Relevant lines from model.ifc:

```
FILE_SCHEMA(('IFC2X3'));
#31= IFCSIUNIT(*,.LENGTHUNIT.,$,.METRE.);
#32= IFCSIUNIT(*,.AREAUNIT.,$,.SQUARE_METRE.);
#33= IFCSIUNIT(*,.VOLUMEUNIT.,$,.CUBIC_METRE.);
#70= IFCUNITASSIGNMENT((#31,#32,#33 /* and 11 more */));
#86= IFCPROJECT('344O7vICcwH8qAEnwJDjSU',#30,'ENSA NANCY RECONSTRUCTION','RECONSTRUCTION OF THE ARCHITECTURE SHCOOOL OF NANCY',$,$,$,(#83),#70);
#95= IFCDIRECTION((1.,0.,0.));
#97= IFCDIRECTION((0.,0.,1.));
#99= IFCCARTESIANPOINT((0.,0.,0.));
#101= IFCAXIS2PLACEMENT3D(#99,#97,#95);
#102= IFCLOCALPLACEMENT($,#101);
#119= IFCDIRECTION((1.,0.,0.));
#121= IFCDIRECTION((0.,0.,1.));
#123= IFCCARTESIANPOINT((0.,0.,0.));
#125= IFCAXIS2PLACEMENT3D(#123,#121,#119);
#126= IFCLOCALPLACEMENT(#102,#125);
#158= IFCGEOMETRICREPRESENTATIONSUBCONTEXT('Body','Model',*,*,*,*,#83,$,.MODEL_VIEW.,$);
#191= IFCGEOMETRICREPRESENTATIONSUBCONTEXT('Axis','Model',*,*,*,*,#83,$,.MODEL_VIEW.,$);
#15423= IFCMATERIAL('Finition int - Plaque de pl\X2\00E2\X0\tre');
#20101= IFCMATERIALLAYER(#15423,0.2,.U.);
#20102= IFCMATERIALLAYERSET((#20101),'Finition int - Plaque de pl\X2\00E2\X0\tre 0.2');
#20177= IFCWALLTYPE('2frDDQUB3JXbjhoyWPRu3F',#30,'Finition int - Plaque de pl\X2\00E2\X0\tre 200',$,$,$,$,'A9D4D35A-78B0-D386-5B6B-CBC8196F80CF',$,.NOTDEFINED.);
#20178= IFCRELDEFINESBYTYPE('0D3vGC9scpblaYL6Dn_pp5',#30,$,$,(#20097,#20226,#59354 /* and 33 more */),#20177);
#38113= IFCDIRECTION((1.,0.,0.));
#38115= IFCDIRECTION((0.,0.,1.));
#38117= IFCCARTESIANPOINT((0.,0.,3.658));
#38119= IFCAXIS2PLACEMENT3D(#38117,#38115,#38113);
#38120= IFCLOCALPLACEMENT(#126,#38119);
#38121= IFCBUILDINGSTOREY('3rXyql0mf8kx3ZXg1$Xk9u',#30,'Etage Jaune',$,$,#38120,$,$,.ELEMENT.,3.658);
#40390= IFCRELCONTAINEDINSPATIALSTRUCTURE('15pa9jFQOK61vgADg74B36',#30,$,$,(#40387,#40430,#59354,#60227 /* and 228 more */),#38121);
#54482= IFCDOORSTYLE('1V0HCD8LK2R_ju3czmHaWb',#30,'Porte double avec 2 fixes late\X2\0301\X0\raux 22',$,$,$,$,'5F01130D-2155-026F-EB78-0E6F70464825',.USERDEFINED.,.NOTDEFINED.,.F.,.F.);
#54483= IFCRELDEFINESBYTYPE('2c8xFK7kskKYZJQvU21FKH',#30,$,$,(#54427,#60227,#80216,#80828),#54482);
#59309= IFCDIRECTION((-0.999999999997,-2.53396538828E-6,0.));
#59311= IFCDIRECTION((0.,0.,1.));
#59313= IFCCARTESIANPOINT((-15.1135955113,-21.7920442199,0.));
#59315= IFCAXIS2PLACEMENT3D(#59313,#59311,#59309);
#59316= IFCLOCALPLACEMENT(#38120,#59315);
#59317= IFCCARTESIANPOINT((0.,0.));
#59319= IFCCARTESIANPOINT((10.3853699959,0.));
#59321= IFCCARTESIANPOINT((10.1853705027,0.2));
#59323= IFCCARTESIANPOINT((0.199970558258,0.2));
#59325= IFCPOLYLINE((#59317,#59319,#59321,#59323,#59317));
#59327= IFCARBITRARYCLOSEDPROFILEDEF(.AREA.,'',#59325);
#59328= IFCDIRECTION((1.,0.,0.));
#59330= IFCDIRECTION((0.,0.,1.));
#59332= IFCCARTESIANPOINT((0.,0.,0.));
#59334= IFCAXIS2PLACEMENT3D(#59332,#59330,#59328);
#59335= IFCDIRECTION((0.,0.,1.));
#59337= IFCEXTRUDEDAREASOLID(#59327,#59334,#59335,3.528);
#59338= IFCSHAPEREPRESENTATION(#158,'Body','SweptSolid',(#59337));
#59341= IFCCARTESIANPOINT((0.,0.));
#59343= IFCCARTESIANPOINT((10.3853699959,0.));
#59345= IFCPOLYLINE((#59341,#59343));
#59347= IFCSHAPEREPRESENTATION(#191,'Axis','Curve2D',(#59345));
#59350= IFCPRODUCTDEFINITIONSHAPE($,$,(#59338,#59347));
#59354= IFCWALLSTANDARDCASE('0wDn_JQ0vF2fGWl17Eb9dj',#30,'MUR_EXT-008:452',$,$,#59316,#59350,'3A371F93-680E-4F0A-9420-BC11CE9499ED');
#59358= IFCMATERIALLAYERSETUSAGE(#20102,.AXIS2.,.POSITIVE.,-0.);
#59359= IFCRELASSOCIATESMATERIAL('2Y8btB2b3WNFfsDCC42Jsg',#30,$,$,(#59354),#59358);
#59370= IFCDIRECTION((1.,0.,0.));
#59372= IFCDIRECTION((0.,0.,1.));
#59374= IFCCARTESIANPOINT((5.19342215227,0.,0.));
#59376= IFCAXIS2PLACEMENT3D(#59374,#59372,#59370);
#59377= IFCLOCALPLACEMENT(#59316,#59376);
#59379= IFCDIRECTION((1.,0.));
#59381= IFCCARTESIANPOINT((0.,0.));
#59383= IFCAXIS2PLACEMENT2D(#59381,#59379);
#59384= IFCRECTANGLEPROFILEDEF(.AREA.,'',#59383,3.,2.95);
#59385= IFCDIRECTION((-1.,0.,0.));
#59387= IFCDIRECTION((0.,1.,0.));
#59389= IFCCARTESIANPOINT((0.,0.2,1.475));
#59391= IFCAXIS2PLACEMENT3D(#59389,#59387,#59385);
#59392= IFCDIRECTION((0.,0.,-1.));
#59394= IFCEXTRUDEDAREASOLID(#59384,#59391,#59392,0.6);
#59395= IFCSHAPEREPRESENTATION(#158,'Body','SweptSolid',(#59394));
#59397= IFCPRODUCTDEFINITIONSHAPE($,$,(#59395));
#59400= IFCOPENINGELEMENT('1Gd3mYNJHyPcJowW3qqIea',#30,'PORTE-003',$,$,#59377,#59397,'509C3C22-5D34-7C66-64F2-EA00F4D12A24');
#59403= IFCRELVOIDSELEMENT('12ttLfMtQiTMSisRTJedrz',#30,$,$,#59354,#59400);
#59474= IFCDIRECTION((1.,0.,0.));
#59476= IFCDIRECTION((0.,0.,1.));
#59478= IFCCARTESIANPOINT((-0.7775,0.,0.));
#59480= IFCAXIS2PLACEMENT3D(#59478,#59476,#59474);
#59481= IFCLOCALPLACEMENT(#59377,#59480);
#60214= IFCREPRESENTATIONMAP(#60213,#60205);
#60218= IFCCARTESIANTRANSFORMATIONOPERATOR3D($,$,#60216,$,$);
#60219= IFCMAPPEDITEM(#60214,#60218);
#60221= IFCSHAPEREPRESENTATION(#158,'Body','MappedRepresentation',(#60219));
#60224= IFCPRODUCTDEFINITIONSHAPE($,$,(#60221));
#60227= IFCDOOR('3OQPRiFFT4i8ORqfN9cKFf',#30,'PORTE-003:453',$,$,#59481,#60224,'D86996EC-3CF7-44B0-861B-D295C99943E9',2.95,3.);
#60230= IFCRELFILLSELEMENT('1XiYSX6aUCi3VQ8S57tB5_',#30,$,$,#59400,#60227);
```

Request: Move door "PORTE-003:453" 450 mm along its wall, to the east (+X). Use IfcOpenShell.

```python
import ifcopenshell
import ifcopenshell.api.geometry
import ifcopenshell.util.placement
import ifcopenshell.util.unit

model = ifcopenshell.open("model.ifc")
unit_scale = ifcopenshell.util.unit.calculate_unit_scale(model)

door = model.by_id(60227)
opening = door.FillsVoids[0].RelatingOpeningElement
wall = opening.VoidsElements[0].RelatingBuildingElement

wall_matrix = ifcopenshell.util.placement.get_local_placement(wall.ObjectPlacement)
shift = wall_matrix[:3, 0] * -0.45 / unit_scale
before = ifcopenshell.util.placement.get_local_placement(door.ObjectPlacement)[:3, 3].copy()

# The door is placed relative to its opening, so it follows when the opening moves.
matrix = ifcopenshell.util.placement.get_local_placement(opening.ObjectPlacement)
matrix[:3, 3] += shift
ifcopenshell.api.geometry.edit_object_placement(
    model, product=opening, matrix=matrix, is_si=False, should_transform_children=True
)

after = ifcopenshell.util.placement.get_local_placement(door.ObjectPlacement)[:3, 3]
print("door moved by", (after - before).round(3) + 0.0)

model.write("model-out.ifc")
```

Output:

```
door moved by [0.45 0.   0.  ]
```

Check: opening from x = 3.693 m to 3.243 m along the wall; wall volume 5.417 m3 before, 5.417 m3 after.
